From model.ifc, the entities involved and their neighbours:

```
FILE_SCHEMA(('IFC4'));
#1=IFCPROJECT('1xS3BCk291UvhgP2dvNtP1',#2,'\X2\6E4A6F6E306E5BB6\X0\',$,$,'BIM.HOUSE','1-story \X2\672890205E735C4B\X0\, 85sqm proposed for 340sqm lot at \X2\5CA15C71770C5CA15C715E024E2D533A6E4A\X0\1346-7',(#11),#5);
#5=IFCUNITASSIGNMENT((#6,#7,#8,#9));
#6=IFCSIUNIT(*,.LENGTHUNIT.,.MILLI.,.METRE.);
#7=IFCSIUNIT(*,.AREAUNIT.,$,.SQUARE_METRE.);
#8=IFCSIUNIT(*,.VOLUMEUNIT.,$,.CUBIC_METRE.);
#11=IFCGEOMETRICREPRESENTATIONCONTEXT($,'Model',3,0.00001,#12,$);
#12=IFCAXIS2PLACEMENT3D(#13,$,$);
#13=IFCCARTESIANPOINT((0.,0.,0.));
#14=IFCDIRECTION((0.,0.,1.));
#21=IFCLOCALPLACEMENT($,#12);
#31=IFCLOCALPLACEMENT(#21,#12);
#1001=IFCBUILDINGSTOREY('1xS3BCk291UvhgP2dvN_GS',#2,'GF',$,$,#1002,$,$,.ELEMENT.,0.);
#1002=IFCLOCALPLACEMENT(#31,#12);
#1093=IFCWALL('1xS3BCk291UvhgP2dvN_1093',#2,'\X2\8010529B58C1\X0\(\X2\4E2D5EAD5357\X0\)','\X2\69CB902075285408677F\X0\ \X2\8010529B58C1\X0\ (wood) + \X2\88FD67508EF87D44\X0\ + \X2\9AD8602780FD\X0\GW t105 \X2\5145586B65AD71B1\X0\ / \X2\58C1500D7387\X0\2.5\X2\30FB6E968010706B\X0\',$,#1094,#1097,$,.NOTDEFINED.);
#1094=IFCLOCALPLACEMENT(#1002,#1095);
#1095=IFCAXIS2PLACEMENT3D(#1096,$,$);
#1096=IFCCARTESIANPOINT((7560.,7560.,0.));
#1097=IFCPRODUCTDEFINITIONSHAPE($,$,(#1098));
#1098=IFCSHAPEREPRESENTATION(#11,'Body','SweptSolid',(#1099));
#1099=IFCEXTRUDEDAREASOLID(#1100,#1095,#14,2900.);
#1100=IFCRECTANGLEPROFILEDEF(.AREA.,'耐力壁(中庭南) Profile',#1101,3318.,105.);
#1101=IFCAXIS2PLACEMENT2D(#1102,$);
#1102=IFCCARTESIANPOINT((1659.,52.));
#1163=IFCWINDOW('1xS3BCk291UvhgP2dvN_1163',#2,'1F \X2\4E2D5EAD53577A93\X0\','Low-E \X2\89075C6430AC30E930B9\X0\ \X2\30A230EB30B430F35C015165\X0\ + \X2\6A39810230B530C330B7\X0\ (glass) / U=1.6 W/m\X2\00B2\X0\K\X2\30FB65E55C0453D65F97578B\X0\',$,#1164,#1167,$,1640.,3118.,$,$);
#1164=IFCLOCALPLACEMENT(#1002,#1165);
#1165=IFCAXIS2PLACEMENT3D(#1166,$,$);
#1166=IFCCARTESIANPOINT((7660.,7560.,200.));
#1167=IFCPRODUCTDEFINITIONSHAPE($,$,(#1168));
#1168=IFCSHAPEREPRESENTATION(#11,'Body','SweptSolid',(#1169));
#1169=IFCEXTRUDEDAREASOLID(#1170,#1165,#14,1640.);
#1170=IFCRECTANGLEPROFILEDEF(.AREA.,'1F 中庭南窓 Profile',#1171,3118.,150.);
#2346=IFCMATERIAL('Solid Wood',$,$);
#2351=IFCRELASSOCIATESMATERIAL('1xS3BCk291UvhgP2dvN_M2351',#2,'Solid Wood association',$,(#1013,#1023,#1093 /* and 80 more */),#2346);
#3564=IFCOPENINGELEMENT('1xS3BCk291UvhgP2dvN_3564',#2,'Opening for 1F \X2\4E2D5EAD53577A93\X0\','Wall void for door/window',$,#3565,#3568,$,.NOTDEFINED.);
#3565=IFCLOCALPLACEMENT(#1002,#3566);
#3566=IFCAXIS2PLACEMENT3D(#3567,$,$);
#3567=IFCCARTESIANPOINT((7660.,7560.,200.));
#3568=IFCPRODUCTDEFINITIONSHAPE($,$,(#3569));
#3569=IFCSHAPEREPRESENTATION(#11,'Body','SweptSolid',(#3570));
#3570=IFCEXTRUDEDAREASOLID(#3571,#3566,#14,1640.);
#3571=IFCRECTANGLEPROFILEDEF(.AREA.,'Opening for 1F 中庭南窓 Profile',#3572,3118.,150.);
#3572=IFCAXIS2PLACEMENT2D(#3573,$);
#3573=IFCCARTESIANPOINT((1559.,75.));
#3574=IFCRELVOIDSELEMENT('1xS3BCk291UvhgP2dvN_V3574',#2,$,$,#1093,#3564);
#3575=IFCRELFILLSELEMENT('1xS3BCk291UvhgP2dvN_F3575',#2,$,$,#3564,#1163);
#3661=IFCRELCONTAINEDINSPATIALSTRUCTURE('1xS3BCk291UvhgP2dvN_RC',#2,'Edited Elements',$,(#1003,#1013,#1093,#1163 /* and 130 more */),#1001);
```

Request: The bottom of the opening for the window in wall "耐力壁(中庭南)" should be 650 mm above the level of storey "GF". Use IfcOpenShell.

```python
import numpy as np
import ifcopenshell
import ifcopenshell.api.geometry
import ifcopenshell.geom
import ifcopenshell.util.element
import ifcopenshell.util.placement
import ifcopenshell.util.shape
import ifcopenshell.util.unit

model = ifcopenshell.open("model.ifc")
unit_scale = ifcopenshell.util.unit.calculate_unit_scale(model)

window = model.by_guid("1xS3BCk291UvhgP2dvN_1163")
opening = window.FillsVoids[0].RelatingOpeningElement
storey = ifcopenshell.util.element.get_container(window, ifc_class="IfcBuildingStorey")
level = ifcopenshell.util.placement.get_local_placement(storey.ObjectPlacement)[2, 3]

# The opening's origin need not be at the sill, so measure its lowest point.
shape = ifcopenshell.geom.create_shape(ifcopenshell.geom.settings(), opening)
bottom = ifcopenshell.util.shape.get_shape_bottom_elevation(shape, shape.geometry) / unit_scale
dz = level + 650.0 - bottom

shift = np.array([0.0, 0.0, dz])
# The window is not placed relative to its opening, so move both.
for product in (opening, window):
    matrix = ifcopenshell.util.placement.get_local_placement(product.ObjectPlacement)
    matrix[:3, 3] += shift
    ifcopenshell.api.geometry.edit_object_placement(model, product=product, matrix=matrix, is_si=False)

print(f"moved by {dz * unit_scale:+.3f} m")

model.write("model_edited.ifc")
```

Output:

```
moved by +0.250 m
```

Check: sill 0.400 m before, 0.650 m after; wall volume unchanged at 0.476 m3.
